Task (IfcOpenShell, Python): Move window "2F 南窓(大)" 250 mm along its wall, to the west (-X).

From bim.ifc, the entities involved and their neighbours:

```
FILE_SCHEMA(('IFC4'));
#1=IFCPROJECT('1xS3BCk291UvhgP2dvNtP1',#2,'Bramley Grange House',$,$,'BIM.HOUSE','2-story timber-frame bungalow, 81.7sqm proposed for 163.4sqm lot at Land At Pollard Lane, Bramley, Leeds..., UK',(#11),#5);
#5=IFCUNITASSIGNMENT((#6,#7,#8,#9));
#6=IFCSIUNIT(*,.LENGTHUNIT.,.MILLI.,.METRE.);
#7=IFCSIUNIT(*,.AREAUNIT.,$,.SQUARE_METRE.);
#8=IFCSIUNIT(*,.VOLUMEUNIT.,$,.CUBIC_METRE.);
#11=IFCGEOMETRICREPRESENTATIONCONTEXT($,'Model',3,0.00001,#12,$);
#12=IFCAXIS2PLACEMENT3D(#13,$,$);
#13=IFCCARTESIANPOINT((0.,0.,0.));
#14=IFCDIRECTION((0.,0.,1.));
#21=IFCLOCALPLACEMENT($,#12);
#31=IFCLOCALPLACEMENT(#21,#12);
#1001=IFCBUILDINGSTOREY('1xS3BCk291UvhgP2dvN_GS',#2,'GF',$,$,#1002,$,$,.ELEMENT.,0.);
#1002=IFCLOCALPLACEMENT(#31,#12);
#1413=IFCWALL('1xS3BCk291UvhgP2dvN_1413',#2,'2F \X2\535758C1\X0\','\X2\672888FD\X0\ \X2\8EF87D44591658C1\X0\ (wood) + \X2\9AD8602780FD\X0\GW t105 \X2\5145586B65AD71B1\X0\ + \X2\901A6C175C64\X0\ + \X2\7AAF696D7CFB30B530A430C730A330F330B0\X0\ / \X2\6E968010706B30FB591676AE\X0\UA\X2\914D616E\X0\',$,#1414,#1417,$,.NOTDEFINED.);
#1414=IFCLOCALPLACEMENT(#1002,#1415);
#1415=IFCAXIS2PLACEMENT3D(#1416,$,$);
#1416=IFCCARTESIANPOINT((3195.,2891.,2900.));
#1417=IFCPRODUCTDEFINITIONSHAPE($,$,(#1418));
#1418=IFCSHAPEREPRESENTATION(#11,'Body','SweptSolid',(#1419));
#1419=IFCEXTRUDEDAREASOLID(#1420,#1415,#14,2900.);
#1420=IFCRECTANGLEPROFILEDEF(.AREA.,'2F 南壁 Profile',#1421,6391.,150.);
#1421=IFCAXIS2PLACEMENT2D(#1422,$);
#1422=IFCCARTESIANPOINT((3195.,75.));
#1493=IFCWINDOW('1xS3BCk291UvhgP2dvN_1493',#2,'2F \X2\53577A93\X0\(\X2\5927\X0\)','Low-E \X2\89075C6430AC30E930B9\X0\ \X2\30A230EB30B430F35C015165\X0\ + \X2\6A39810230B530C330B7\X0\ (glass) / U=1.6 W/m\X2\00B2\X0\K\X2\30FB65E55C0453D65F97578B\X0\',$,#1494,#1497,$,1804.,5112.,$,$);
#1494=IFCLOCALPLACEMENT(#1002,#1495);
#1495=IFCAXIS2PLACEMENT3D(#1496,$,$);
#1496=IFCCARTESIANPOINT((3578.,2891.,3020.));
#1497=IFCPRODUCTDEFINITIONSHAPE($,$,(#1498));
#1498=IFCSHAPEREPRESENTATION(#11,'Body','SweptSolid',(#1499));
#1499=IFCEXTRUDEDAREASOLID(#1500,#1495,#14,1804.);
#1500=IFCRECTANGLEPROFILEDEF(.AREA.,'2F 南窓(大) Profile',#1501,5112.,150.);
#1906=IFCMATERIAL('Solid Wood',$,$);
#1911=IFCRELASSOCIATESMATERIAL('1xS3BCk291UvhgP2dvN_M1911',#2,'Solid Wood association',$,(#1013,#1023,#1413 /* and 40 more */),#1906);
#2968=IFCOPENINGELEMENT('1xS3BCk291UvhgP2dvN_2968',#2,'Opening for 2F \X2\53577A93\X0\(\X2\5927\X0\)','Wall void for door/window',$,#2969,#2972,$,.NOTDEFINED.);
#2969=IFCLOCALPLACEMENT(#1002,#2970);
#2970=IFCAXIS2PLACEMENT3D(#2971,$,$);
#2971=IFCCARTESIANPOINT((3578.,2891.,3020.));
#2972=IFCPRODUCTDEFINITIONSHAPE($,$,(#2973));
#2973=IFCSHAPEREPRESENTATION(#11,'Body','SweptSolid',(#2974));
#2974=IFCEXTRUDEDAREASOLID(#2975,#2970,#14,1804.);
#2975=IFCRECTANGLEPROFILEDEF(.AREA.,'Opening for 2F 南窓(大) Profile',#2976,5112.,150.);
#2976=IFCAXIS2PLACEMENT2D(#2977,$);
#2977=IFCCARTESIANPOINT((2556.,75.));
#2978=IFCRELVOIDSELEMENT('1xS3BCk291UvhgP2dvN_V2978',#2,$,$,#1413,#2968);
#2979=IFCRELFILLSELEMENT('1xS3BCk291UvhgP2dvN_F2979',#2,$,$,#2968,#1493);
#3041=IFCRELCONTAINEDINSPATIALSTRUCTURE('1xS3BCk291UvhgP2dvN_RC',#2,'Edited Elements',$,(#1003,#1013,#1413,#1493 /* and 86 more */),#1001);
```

```python
import ifcopenshell
import ifcopenshell.api.geometry
import ifcopenshell.util.placement
import ifcopenshell.util.unit

model = ifcopenshell.open("bim.ifc")
unit_scale = ifcopenshell.util.unit.calculate_unit_scale(model)

window = model.by_id(1493)
opening = window.FillsVoids[0].RelatingOpeningElement
wall = opening.VoidsElements[0].RelatingBuildingElement

wall_matrix = ifcopenshell.util.placement.get_local_placement(wall.ObjectPlacement)
shift = wall_matrix[:3, 0] * -0.25 / unit_scale
before = ifcopenshell.util.placement.get_local_placement(window.ObjectPlacement)[:3, 3].copy()

# The window is not placed relative to its opening, so move both.
for product in (opening, window):
    matrix = ifcopenshell.util.placement.get_local_placement(product.ObjectPlacement)
    matrix[:3, 3] += shift
    ifcopenshell.api.geometry.edit_object_placement(model, product=product, matrix=matrix, is_si=False)

after = ifcopenshell.util.placement.get_local_placement(window.ObjectPlacement)[:3, 3]
print("window moved by", (after - before).round(3) + 0.0)

model.write("bim-out.ifc")
```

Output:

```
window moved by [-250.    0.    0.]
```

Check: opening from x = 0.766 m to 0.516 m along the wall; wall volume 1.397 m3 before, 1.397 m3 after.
